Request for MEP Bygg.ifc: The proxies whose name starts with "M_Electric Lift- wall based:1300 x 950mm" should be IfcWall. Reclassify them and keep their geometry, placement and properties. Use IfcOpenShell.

First a look at what the model holds.

```python
import re

import ifcopenshell

model = ifcopenshell.open("MEP Bygg.ifc")
print(model.schema)
seen = {}
for e in model.by_type("IfcBuildingElementProxy"):
    name = re.sub(r":\d+(:\d+)?$", "", e.Name or "")  # drop the element id that some exporters append
    seen[name] = seen.get(name, 0) + 1
for name, count in sorted(seen.items()):
    print(count, "x", name)
```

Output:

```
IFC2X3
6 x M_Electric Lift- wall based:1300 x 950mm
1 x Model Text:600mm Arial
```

```python
import ifcopenshell
import ifcopenshell.api.root

model = ifcopenshell.open("MEP Bygg.ifc")

proxies = [e.id() for e in model.by_type("IfcBuildingElementProxy") if (e.Name or "").startswith("M_Electric Lift- wall based:1300 x 950mm")]
for step_id in proxies:
    proxy = model.by_id(step_id)
    ifcopenshell.api.root.reassign_class(model, product=proxy, ifc_class="IfcWall")

print(sum(model.by_id(i).is_a("IfcWall") for i in proxies), "reclassified")

model.write("MEP Bygg_v2.ifc")
```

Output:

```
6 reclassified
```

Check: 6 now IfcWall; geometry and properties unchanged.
